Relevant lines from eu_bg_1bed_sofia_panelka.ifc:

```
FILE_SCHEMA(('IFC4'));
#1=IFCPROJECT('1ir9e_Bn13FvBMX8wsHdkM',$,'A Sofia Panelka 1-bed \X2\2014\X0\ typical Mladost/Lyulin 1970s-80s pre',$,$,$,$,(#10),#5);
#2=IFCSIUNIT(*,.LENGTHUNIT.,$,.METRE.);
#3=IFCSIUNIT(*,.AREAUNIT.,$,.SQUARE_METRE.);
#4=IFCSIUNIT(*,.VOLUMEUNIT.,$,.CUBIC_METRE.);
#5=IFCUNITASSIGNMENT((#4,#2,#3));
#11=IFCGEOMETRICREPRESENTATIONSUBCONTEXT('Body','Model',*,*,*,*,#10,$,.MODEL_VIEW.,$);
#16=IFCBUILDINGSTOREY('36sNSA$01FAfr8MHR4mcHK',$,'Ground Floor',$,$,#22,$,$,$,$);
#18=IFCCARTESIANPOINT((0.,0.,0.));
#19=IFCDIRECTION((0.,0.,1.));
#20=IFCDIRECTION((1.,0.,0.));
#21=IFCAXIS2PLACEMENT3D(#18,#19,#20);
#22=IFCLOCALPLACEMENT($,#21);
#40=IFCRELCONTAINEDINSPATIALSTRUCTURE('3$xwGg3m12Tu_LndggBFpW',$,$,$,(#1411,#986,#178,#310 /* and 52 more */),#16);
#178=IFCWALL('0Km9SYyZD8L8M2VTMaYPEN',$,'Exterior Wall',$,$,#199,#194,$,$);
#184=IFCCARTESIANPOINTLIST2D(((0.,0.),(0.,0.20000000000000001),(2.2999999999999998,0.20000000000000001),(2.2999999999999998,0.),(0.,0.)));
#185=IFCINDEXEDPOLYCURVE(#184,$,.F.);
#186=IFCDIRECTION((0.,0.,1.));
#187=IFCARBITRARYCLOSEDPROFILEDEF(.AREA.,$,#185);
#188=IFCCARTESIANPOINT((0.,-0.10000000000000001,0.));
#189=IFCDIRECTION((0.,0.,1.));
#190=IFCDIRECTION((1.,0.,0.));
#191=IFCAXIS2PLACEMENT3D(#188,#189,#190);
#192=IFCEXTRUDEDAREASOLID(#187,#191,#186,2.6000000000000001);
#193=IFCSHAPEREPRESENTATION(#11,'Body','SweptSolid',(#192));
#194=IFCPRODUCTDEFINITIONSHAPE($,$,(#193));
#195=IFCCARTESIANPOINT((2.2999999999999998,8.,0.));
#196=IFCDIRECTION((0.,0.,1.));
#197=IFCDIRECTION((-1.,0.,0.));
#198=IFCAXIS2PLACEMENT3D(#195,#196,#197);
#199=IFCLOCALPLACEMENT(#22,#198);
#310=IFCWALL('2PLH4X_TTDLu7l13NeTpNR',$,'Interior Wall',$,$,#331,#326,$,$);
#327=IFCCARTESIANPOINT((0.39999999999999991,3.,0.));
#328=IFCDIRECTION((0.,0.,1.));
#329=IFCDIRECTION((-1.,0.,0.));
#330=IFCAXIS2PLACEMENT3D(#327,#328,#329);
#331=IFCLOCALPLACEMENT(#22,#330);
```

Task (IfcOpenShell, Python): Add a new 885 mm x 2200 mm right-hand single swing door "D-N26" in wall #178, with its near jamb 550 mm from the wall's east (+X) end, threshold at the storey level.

```python
import numpy as np
import ifcopenshell
import ifcopenshell.api.feature
import ifcopenshell.api.geometry
import ifcopenshell.api.root
import ifcopenshell.api.spatial
import ifcopenshell.geom
import ifcopenshell.util.element
import ifcopenshell.util.placement
import ifcopenshell.util.representation
import ifcopenshell.util.shape
import ifcopenshell.util.unit

model = ifcopenshell.open("eu_bg_1bed_sofia_panelka.ifc")
unit_scale = ifcopenshell.util.unit.calculate_unit_scale(model)
settings = ifcopenshell.geom.settings()


def volume(element):
    """Net volume in cubic metres, openings subtracted."""
    shape = ifcopenshell.geom.create_shape(settings, element)
    return ifcopenshell.util.shape.get_volume(shape.geometry)


wall = model.by_guid("0Km9SYyZD8L8M2VTMaYPEN")
storey = ifcopenshell.util.element.get_container(wall, ifc_class="IfcBuildingStorey")
context = ifcopenshell.util.representation.get_context(model, "Model", "Body", "MODEL_VIEW")
before = volume(wall)

width, height, from_end, sill = 0.885, 2.2, 0.55, 0.0  # metres

# The wall runs along its own X axis, and the end named is its -X end.
wall_shape = ifcopenshell.geom.create_shape(settings, wall)
x, y, z = ifcopenshell.util.shape.get_vertices(wall_shape.geometry).T
start = x.min() + from_end
face, thickness = float(y.min()), float(y.max() - y.min())
wall_matrix = ifcopenshell.util.placement.get_local_placement(wall.ObjectPlacement)
level = ifcopenshell.util.placement.get_local_placement(storey.ObjectPlacement)[2, 3]


def in_wall(x, y):
    """Placement at x, y metres in the wall's axes, at sill height."""
    matrix = wall_matrix.copy()
    matrix[:, 3] = wall_matrix @ np.array([x / unit_scale, y / unit_scale, 0.0, 1.0])
    matrix[2, 3] = level + sill / unit_scale
    return matrix


# Opening: a box that overshoots both wall faces by 50 mm.
opening = ifcopenshell.api.root.create_entity(model, ifc_class="IfcOpeningElement", predefined_type="OPENING")
box = ifcopenshell.api.geometry.add_wall_representation(
    model, context=context, length=width, height=height, thickness=thickness + 0.1
)
ifcopenshell.api.geometry.assign_representation(model, product=opening, representation=box)
ifcopenshell.api.geometry.edit_object_placement(model, product=opening, matrix=in_wall(start, face - 0.05), is_si=False)
ifcopenshell.api.feature.add_feature(model, feature=opening, element=wall)

door = ifcopenshell.api.root.create_entity(model, ifc_class="IfcDoor", name="D-N26", predefined_type="DOOR")
door.OverallWidth, door.OverallHeight = width / unit_scale, height / unit_scale
door.OperationType = "SINGLE_SWING_RIGHT"
body = ifcopenshell.api.geometry.add_door_representation(
    model,
    context=context,
    overall_width=door.OverallWidth,
    overall_height=door.OverallHeight,
    operation_type="SINGLE_SWING_RIGHT",
    lining_properties={"LiningDepth": thickness / unit_scale, "ThresholdDepth": thickness / unit_scale},
)
ifcopenshell.api.geometry.assign_representation(model, product=door, representation=body)
ifcopenshell.api.spatial.assign_container(model, products=[door], relating_structure=storey)
ifcopenshell.api.feature.add_filling(model, opening=opening, element=door)

# The lining spans the wall, so the door starts at the wall face.
ifcopenshell.api.geometry.edit_object_placement(model, product=door, matrix=in_wall(start, face), is_si=False)

after = volume(wall)

print(f"wall volume {before:.3f} -> {after:.3f} m3")

model.write("eu_bg_1bed_sofia_panelka_updated.ifc")
```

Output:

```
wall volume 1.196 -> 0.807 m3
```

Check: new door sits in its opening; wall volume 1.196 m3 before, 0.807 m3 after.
